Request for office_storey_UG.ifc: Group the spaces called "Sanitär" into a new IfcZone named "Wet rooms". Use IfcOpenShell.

First a look at what the model holds.

```python
import ifcopenshell

model = ifcopenshell.open("office_storey_UG.ifc")
print(model.schema)
seen = {}
for space in model.by_type("IfcSpace"):
    seen[space.LongName] = seen.get(space.LongName, 0) + 1
for name, count in sorted(seen.items(), key=str):
    print(count, "x", name)
print("zones:", [z.Name for z in model.by_type("IfcZone")][:20])
```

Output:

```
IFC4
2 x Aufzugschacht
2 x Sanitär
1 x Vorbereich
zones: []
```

```python
import ifcopenshell
import ifcopenshell.api.group
import ifcopenshell.api.root

model = ifcopenshell.open("office_storey_UG.ifc")

names = {"Sanitär"}
spaces = [s for s in model.by_type("IfcSpace") if s.LongName in names]

zone = ifcopenshell.api.root.create_entity(model, ifc_class="IfcZone", name="Wet rooms")
ifcopenshell.api.group.assign_group(model, products=spaces, group=zone)
print(len(spaces), "spaces in", zone.Name)

model.write("office_storey_UG_v2.ifc")
```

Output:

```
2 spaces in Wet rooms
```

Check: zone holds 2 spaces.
